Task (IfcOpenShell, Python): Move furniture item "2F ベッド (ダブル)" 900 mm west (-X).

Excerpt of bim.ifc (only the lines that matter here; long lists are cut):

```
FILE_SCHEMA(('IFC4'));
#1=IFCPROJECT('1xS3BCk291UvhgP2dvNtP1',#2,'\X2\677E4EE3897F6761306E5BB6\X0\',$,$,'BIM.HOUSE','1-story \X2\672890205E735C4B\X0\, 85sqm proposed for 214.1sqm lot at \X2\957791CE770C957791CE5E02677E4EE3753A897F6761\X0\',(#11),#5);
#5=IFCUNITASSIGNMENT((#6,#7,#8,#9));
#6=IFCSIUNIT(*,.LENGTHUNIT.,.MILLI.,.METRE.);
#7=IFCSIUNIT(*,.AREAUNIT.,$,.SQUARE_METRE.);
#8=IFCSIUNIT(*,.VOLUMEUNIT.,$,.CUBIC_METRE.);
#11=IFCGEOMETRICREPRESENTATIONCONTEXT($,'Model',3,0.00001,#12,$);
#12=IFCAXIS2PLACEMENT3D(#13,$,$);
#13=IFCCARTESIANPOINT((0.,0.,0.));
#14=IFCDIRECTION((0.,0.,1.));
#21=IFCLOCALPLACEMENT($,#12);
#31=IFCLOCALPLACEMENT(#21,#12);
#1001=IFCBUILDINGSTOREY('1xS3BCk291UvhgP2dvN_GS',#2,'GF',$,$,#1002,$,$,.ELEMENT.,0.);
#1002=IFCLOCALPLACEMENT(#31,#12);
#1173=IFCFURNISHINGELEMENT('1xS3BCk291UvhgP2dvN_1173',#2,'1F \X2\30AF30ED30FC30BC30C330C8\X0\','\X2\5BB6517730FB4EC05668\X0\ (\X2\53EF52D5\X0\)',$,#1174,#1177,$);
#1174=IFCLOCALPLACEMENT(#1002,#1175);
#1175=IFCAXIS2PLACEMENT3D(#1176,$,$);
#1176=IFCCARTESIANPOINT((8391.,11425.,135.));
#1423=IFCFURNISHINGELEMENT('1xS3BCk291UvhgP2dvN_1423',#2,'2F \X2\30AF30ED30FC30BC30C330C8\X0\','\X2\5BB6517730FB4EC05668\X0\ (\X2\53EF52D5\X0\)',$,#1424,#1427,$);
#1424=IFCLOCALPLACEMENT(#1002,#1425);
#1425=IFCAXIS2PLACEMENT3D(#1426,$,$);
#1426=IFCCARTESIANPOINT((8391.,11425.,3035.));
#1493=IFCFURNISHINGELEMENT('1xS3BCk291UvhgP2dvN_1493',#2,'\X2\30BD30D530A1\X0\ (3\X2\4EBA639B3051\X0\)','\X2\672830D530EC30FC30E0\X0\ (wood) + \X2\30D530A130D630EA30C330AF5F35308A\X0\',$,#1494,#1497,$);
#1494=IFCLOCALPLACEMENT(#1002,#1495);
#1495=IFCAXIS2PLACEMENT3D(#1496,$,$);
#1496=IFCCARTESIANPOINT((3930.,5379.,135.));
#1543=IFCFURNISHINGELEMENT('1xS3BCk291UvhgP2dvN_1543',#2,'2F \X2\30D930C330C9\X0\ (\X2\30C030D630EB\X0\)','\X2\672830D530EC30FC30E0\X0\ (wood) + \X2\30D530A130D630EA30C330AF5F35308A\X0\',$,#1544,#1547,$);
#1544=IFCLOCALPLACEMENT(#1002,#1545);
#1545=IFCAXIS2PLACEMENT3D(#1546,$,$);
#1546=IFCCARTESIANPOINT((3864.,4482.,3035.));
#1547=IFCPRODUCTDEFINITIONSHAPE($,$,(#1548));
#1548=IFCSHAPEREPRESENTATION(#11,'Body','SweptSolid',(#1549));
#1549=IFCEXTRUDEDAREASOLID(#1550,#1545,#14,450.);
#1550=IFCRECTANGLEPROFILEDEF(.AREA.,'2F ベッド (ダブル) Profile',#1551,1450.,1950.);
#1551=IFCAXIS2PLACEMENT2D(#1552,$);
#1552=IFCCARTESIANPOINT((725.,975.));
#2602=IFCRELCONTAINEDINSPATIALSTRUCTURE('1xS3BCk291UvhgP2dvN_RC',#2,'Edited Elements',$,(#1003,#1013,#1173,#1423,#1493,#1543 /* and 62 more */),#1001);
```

```python
import ifcopenshell
import ifcopenshell.api.geometry
import ifcopenshell.util.placement
import ifcopenshell.util.unit

model = ifcopenshell.open("bim.ifc")
unit_scale = ifcopenshell.util.unit.calculate_unit_scale(model)

item = model.by_guid("1xS3BCk291UvhgP2dvN_1543")
matrix = ifcopenshell.util.placement.get_local_placement(item.ObjectPlacement)
matrix[0, 3] -= 0.9 / unit_scale
ifcopenshell.api.geometry.edit_object_placement(model, product=item, matrix=matrix, is_si=False)

print(ifcopenshell.util.placement.get_local_placement(item.ObjectPlacement).round(3) + 0.0)

model.write("bim-out.ifc")
```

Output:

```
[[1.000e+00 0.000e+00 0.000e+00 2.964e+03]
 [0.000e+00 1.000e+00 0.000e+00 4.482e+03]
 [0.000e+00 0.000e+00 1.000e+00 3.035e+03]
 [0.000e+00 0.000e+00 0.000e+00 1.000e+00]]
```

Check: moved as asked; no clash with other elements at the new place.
